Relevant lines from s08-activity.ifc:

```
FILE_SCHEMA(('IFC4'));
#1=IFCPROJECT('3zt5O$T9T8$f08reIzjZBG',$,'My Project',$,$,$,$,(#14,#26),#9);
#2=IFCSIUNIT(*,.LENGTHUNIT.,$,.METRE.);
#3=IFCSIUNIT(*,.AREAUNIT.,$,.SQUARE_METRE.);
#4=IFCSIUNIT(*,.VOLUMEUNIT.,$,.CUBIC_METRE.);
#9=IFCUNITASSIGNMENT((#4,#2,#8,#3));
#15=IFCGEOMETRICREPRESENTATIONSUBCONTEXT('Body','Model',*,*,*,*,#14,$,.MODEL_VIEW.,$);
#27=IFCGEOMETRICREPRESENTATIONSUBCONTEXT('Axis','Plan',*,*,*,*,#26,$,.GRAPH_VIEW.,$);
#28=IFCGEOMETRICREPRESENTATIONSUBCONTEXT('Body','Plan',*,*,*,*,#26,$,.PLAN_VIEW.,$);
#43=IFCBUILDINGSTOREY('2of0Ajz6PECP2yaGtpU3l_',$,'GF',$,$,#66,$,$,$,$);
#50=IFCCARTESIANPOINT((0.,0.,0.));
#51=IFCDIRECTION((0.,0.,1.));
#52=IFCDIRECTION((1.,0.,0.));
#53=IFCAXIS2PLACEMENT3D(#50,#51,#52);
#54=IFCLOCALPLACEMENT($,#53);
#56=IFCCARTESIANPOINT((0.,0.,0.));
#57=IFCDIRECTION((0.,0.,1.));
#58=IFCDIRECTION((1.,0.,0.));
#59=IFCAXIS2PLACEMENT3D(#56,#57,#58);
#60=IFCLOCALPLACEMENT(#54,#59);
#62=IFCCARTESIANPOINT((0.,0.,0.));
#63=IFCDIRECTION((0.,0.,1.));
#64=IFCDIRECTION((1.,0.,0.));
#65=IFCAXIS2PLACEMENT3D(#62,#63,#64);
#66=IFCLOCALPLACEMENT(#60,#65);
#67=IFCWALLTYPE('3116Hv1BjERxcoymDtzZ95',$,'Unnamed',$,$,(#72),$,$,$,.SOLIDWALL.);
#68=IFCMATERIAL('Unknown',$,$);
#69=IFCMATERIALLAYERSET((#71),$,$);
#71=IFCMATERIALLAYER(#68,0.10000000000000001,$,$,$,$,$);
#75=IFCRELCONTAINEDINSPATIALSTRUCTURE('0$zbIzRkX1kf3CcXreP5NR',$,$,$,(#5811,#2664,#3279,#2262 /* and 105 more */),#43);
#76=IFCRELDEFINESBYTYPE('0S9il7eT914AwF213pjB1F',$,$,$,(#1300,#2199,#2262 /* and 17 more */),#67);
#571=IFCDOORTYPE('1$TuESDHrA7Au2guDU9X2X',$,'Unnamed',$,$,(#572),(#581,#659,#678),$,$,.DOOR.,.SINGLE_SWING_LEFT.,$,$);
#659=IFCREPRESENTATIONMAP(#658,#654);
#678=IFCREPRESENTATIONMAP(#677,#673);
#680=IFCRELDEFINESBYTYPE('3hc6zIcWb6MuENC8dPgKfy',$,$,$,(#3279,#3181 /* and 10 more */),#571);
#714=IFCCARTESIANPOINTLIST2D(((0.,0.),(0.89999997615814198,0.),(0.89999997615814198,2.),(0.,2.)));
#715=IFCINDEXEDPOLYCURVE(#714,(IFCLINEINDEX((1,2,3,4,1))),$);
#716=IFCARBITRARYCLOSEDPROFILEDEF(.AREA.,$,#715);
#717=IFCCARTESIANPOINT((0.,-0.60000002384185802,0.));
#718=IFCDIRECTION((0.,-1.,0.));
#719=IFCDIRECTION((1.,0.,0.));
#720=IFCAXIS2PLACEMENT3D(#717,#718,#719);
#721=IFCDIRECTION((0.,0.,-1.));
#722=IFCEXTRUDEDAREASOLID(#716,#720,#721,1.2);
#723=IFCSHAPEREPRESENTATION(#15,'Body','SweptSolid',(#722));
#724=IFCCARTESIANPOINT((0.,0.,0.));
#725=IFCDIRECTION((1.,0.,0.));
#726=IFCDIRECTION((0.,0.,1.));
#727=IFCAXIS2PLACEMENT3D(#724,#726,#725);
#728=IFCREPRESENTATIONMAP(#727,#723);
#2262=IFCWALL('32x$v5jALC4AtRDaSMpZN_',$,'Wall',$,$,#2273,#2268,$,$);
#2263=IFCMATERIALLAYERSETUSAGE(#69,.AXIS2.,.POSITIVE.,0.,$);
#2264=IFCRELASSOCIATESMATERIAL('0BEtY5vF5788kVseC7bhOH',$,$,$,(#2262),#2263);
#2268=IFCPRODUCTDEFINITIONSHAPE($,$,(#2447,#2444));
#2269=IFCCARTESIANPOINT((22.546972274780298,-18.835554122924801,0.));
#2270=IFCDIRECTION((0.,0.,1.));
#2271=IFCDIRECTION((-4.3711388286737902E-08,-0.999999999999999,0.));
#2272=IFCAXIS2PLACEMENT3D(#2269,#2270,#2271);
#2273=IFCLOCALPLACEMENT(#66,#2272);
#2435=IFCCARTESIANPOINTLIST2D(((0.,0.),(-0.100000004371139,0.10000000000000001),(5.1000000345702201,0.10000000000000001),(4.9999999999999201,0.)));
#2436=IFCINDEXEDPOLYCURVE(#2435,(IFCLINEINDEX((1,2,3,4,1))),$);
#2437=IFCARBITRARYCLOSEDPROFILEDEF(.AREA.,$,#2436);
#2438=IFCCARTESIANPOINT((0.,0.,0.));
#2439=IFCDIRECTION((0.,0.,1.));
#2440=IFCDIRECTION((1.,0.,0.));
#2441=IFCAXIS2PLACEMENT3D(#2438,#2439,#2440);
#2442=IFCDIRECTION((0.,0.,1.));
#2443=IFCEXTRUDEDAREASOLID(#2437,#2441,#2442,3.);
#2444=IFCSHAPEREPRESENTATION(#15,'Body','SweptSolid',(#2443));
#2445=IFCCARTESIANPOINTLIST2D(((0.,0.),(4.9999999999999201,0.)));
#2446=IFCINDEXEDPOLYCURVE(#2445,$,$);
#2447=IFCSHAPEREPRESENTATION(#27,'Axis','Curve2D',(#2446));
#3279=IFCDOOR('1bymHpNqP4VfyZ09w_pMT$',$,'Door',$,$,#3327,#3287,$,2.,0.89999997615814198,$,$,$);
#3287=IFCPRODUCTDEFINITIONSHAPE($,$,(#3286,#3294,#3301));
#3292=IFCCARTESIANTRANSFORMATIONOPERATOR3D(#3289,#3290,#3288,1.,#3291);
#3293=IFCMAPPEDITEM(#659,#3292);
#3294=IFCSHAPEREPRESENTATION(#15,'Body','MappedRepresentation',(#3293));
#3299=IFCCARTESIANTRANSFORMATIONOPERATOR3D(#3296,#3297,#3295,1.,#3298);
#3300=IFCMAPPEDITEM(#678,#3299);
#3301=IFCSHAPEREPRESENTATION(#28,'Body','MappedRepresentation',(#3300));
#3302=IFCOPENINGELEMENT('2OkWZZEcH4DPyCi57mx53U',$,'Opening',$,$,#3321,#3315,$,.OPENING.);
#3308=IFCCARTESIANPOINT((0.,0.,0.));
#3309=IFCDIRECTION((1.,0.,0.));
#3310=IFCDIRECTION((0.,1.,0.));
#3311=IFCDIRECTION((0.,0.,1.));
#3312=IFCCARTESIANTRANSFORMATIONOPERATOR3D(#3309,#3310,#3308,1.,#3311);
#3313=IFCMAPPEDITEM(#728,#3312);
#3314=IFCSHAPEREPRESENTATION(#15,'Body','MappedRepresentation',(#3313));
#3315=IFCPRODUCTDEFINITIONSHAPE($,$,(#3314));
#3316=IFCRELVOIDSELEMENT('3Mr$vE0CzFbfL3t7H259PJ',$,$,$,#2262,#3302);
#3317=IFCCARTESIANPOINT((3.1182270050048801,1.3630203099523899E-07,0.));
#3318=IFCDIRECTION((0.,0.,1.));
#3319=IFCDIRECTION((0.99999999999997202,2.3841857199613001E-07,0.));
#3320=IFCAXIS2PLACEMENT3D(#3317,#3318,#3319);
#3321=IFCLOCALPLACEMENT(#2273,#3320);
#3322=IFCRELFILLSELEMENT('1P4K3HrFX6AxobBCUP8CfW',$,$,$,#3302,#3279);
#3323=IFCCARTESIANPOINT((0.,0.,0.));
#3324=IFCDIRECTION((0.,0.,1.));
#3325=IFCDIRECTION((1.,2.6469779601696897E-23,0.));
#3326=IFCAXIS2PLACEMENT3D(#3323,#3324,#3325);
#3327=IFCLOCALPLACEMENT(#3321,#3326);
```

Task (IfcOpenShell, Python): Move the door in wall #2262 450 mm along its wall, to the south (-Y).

```python
import ifcopenshell
import ifcopenshell.api.geometry
import ifcopenshell.util.placement

model = ifcopenshell.open("s08-activity.ifc")

door = model.by_guid("1bymHpNqP4VfyZ09w_pMT$")
opening = door.FillsVoids[0].RelatingOpeningElement
wall = opening.VoidsElements[0].RelatingBuildingElement

wall_matrix = ifcopenshell.util.placement.get_local_placement(wall.ObjectPlacement)
shift = wall_matrix[:3, 0] * 0.45
before = ifcopenshell.util.placement.get_local_placement(door.ObjectPlacement)[:3, 3].copy()

# The door is placed relative to its opening, so it follows when the opening moves.
matrix = ifcopenshell.util.placement.get_local_placement(opening.ObjectPlacement)
matrix[:3, 3] += shift
ifcopenshell.api.geometry.edit_object_placement(
    model, product=opening, matrix=matrix, is_si=False, should_transform_children=True
)

after = ifcopenshell.util.placement.get_local_placement(door.ObjectPlacement)[:3, 3]
print("door moved by", (after - before).round(3) + 0.0)

model.write("s08-activity-out.ifc")
```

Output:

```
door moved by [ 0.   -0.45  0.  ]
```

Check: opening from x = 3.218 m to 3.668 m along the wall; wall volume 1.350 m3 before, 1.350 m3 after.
